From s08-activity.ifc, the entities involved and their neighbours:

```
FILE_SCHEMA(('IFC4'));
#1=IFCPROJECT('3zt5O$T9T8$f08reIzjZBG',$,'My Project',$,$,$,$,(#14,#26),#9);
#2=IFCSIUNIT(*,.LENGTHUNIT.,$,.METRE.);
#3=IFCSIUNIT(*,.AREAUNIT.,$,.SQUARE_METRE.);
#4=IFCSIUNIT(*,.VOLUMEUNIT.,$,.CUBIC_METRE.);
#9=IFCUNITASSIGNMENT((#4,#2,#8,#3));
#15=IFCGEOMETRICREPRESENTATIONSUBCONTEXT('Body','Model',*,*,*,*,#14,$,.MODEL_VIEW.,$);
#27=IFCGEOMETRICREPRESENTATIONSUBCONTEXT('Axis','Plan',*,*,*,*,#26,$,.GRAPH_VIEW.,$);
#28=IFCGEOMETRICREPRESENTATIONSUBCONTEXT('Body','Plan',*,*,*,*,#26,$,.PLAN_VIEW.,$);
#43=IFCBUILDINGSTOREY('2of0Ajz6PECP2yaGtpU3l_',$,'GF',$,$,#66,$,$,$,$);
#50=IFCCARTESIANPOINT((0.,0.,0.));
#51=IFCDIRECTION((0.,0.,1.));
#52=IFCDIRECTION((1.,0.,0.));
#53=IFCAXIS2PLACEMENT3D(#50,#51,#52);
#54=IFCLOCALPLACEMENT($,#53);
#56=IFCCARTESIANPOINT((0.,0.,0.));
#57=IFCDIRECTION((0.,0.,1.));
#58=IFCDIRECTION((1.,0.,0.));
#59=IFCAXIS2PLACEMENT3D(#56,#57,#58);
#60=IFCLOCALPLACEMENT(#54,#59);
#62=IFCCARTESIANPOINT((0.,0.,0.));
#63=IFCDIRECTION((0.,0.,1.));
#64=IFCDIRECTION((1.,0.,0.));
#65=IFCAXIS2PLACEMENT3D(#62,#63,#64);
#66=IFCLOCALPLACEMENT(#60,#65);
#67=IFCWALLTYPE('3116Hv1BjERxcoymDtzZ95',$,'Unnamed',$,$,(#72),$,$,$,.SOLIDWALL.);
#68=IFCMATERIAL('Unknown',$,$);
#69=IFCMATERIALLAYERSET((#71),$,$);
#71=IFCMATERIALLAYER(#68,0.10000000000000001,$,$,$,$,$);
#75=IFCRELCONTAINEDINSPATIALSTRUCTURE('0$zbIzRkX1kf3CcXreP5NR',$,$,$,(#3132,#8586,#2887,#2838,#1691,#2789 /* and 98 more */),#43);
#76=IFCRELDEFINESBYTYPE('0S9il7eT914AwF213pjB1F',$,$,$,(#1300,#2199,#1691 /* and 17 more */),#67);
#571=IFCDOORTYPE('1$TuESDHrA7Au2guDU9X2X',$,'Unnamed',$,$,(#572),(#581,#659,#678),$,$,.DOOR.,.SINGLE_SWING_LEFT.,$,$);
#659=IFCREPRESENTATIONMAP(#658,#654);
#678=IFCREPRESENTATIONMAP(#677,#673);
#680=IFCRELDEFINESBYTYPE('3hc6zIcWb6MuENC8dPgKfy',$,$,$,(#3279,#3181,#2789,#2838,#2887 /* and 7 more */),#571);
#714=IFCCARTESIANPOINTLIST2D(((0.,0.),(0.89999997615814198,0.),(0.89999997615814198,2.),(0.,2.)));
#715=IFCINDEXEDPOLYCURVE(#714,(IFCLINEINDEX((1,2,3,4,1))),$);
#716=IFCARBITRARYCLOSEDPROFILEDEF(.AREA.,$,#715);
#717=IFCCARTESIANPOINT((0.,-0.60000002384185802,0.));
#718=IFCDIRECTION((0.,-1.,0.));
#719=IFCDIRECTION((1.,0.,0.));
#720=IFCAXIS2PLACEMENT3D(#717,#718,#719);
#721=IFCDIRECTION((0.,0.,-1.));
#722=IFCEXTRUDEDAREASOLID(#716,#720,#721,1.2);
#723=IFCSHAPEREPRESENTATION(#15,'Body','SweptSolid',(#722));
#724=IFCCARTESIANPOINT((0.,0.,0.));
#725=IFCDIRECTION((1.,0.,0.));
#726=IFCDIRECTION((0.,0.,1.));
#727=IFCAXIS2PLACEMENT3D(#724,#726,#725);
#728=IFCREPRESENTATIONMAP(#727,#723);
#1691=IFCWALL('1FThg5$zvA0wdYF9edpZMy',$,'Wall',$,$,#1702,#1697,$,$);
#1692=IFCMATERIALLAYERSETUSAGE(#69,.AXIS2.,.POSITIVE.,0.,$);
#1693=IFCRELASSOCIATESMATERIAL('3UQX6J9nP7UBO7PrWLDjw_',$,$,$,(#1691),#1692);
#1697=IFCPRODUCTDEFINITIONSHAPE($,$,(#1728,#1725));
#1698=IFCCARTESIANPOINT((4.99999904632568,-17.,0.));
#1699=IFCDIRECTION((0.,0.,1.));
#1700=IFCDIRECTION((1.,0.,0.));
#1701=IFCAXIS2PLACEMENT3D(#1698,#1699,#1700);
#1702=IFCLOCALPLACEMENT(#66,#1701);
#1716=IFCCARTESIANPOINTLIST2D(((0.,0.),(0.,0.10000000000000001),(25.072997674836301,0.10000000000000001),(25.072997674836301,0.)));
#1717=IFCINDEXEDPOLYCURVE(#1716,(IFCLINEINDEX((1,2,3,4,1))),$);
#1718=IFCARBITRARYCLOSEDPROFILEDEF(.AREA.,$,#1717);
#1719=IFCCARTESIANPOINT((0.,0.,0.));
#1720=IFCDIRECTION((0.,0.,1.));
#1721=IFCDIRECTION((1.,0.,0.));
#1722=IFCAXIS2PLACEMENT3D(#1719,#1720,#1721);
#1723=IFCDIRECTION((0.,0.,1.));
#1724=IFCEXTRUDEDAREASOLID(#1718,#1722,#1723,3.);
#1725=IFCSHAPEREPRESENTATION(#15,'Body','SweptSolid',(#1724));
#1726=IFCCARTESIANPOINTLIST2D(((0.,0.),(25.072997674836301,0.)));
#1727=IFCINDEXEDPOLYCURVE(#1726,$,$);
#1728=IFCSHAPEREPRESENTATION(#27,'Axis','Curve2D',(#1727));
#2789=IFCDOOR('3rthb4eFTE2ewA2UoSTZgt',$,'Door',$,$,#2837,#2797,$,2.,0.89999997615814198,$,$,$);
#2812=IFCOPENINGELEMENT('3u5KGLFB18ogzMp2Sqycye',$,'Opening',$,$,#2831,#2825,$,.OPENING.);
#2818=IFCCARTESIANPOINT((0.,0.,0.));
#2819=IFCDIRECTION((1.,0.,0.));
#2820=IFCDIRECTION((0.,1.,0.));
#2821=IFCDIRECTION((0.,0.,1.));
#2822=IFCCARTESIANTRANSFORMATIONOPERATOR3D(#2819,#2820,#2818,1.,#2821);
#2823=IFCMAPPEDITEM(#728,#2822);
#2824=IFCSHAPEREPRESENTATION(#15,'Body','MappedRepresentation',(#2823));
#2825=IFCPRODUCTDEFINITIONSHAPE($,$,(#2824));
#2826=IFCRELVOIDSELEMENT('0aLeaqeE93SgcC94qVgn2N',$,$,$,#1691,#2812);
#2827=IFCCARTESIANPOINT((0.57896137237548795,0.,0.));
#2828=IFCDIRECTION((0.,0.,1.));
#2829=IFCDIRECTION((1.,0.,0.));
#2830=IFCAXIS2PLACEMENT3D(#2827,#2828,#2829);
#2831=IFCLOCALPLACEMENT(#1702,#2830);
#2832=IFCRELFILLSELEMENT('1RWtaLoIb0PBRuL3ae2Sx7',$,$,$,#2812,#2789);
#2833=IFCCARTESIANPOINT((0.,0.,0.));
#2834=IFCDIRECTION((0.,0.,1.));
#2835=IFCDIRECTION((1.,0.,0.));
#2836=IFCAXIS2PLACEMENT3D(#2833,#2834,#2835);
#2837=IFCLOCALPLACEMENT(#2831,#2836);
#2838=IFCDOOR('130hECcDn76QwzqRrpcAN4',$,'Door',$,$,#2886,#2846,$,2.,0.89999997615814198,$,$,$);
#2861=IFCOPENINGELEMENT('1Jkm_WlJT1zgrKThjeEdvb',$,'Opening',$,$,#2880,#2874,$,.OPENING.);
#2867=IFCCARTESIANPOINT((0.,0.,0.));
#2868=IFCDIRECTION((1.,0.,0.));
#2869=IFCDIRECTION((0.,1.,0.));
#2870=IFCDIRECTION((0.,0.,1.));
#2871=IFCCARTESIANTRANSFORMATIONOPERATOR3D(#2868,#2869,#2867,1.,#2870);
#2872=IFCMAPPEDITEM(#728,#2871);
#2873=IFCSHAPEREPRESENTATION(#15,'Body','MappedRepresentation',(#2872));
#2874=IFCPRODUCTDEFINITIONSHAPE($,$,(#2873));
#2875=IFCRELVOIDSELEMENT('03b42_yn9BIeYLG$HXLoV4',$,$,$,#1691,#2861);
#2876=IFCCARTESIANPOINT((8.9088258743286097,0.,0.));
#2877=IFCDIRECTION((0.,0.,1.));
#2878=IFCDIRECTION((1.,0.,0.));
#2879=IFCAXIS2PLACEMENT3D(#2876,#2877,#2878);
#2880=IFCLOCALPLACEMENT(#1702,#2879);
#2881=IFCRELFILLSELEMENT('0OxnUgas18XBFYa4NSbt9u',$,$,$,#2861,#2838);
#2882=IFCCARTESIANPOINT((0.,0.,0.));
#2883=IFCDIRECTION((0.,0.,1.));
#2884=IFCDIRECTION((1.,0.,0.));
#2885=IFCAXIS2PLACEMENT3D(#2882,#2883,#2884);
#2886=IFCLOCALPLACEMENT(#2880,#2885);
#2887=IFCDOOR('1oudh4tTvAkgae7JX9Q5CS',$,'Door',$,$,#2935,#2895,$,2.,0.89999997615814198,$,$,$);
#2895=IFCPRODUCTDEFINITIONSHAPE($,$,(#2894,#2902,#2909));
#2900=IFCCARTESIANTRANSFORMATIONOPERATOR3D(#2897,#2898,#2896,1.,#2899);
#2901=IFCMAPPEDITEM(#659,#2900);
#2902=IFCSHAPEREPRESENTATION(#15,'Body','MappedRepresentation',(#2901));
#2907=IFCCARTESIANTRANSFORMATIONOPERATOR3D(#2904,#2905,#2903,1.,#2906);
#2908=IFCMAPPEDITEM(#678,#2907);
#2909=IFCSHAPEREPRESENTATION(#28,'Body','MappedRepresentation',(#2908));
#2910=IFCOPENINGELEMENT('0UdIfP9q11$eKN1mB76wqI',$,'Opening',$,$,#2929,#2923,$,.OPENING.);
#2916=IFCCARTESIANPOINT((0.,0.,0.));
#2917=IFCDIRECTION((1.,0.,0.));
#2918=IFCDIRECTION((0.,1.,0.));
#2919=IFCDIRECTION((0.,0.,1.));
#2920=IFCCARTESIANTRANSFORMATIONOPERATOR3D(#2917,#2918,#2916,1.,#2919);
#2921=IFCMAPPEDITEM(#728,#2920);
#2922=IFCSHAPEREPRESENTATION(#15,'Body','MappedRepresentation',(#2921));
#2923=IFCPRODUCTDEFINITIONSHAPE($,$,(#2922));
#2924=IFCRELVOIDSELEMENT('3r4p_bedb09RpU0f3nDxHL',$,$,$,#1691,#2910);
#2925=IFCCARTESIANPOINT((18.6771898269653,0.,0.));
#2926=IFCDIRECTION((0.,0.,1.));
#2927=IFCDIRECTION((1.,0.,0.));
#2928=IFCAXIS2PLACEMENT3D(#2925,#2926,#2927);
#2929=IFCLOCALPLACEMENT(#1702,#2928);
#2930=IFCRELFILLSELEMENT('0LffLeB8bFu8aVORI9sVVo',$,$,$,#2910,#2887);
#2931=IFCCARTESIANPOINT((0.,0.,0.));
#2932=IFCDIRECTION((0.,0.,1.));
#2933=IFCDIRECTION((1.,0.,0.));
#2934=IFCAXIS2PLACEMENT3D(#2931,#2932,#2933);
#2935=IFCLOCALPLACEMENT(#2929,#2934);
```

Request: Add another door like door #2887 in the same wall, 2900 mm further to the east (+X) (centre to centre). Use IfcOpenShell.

```python
import ifcopenshell
import ifcopenshell.api.feature
import ifcopenshell.api.geometry
import ifcopenshell.api.root
import ifcopenshell.geom
import ifcopenshell.util.element
import ifcopenshell.util.placement
import ifcopenshell.util.shape
import ifcopenshell.util.unit

model = ifcopenshell.open("s08-activity.ifc")
unit_scale = ifcopenshell.util.unit.calculate_unit_scale(model)
settings = ifcopenshell.geom.settings()


def volume(element):
    """Net volume in cubic metres, openings subtracted."""
    shape = ifcopenshell.geom.create_shape(settings, element)
    return ifcopenshell.util.shape.get_volume(shape.geometry)


door = model.by_id(2887)
opening = door.FillsVoids[0].RelatingOpeningElement
wall = opening.VoidsElements[0].RelatingBuildingElement
before = volume(wall)
shift = ifcopenshell.util.placement.get_local_placement(wall.ObjectPlacement)[:3, 0] * 2.9 / unit_scale

# copy_class copies the void relationship, type, container and properties, but no geometry.
new_opening = ifcopenshell.api.root.copy_class(model, product=opening)
new_opening.Representation = ifcopenshell.util.element.copy_deep(
    model, opening.Representation, exclude=["IfcGeometricRepresentationContext", "IfcRepresentationMap"]
)
new_door = ifcopenshell.api.root.copy_class(model, product=door)
new_door.Representation = ifcopenshell.util.element.copy_deep(
    model, door.Representation, exclude=["IfcGeometricRepresentationContext", "IfcRepresentationMap"]
)
ifcopenshell.api.feature.add_filling(model, opening=new_opening, element=new_door)

for old, new in ((opening, new_opening), (door, new_door)):
    matrix = ifcopenshell.util.placement.get_local_placement(old.ObjectPlacement)
    matrix[:3, 3] += shift
    ifcopenshell.api.geometry.edit_object_placement(model, product=new, matrix=matrix, is_si=False)

after = volume(wall)

print(f"wall volume {before:.3f} -> {after:.3f} m3")

model.write("s08-activity_updated.ifc")
```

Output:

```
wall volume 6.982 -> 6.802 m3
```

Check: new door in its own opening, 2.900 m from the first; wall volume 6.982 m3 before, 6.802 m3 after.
